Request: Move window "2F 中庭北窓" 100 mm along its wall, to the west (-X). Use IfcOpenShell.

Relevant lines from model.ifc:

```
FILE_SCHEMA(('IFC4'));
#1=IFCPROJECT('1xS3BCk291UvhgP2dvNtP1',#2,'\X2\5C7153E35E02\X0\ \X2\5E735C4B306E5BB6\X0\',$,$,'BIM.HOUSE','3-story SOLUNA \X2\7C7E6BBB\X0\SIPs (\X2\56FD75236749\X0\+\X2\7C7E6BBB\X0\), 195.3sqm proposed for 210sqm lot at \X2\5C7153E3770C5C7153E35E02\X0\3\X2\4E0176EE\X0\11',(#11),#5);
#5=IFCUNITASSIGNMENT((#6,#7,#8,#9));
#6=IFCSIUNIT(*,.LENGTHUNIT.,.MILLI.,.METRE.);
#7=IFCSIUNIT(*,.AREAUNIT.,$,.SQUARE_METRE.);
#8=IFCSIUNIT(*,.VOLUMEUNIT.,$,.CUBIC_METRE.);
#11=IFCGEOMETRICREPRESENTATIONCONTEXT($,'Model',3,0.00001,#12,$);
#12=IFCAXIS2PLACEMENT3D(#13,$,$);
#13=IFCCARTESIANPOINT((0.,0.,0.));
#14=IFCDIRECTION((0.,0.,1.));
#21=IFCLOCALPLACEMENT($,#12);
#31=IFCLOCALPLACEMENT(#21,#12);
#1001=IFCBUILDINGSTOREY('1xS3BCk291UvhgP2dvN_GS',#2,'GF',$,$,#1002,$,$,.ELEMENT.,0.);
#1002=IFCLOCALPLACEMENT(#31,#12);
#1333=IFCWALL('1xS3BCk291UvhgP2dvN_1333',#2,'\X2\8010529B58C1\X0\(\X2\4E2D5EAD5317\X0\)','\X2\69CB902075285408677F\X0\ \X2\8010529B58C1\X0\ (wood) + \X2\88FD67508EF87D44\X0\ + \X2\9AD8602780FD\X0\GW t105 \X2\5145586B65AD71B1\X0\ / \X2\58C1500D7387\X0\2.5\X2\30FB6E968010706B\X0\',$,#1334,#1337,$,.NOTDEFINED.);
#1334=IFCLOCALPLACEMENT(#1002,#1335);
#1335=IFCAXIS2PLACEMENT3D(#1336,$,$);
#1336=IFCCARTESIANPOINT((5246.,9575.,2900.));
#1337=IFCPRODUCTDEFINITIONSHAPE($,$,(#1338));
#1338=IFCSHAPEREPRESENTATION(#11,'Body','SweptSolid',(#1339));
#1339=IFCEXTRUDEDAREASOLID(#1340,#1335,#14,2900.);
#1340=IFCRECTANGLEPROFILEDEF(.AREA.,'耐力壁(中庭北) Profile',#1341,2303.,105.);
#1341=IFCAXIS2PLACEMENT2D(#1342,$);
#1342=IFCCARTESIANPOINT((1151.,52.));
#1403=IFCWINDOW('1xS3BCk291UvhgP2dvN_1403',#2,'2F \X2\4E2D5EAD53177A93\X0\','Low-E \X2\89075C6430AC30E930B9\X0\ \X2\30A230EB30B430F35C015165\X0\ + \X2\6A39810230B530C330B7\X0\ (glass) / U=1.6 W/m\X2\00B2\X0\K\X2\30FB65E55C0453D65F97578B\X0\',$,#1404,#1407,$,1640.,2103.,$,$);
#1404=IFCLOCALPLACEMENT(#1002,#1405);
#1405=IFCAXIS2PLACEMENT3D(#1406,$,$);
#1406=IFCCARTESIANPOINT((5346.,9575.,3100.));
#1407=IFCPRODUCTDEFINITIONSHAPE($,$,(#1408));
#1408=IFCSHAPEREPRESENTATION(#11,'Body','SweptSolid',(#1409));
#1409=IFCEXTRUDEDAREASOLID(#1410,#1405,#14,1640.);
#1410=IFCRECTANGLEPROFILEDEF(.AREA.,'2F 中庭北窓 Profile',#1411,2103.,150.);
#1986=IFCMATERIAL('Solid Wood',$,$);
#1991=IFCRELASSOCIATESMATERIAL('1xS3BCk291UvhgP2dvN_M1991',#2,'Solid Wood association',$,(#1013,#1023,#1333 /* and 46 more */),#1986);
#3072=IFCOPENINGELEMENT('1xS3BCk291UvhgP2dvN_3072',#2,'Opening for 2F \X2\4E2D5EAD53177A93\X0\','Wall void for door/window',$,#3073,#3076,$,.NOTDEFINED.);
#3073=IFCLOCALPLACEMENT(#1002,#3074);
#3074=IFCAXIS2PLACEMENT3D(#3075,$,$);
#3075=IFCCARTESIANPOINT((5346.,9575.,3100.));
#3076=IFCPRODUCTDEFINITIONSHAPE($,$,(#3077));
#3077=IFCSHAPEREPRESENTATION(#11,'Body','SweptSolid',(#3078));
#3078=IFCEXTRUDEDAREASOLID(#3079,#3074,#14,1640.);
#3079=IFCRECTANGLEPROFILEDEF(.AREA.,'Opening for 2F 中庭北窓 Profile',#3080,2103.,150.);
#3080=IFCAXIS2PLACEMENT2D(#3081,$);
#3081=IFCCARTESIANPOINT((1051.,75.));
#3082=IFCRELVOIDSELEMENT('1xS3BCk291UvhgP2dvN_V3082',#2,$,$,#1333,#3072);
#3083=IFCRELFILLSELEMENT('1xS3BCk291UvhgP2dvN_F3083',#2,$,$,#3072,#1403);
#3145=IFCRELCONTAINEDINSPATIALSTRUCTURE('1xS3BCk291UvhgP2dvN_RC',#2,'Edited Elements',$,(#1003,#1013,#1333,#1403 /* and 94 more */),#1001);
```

```python
import ifcopenshell
import ifcopenshell.api.geometry
import ifcopenshell.util.placement

model = ifcopenshell.open("model.ifc")

window = model.by_guid("1xS3BCk291UvhgP2dvN_1403")
opening = window.FillsVoids[0].RelatingOpeningElement
wall = opening.VoidsElements[0].RelatingBuildingElement

wall_matrix = ifcopenshell.util.placement.get_local_placement(wall.ObjectPlacement)
shift = wall_matrix[:3, 0] * -100.0
before = ifcopenshell.util.placement.get_local_placement(window.ObjectPlacement)[:3, 3].copy()

# The window is not placed relative to its opening, so move both.
for product in (opening, window):
    matrix = ifcopenshell.util.placement.get_local_placement(product.ObjectPlacement)
    matrix[:3, 3] += shift
    ifcopenshell.api.geometry.edit_object_placement(model, product=product, matrix=matrix, is_si=False)

after = ifcopenshell.util.placement.get_local_placement(window.ObjectPlacement)[:3, 3]
print("window moved by", (after - before).round(3) + 0.0)

model.write("model_rev.ifc")
```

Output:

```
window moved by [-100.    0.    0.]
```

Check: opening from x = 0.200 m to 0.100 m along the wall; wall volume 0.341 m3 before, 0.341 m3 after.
